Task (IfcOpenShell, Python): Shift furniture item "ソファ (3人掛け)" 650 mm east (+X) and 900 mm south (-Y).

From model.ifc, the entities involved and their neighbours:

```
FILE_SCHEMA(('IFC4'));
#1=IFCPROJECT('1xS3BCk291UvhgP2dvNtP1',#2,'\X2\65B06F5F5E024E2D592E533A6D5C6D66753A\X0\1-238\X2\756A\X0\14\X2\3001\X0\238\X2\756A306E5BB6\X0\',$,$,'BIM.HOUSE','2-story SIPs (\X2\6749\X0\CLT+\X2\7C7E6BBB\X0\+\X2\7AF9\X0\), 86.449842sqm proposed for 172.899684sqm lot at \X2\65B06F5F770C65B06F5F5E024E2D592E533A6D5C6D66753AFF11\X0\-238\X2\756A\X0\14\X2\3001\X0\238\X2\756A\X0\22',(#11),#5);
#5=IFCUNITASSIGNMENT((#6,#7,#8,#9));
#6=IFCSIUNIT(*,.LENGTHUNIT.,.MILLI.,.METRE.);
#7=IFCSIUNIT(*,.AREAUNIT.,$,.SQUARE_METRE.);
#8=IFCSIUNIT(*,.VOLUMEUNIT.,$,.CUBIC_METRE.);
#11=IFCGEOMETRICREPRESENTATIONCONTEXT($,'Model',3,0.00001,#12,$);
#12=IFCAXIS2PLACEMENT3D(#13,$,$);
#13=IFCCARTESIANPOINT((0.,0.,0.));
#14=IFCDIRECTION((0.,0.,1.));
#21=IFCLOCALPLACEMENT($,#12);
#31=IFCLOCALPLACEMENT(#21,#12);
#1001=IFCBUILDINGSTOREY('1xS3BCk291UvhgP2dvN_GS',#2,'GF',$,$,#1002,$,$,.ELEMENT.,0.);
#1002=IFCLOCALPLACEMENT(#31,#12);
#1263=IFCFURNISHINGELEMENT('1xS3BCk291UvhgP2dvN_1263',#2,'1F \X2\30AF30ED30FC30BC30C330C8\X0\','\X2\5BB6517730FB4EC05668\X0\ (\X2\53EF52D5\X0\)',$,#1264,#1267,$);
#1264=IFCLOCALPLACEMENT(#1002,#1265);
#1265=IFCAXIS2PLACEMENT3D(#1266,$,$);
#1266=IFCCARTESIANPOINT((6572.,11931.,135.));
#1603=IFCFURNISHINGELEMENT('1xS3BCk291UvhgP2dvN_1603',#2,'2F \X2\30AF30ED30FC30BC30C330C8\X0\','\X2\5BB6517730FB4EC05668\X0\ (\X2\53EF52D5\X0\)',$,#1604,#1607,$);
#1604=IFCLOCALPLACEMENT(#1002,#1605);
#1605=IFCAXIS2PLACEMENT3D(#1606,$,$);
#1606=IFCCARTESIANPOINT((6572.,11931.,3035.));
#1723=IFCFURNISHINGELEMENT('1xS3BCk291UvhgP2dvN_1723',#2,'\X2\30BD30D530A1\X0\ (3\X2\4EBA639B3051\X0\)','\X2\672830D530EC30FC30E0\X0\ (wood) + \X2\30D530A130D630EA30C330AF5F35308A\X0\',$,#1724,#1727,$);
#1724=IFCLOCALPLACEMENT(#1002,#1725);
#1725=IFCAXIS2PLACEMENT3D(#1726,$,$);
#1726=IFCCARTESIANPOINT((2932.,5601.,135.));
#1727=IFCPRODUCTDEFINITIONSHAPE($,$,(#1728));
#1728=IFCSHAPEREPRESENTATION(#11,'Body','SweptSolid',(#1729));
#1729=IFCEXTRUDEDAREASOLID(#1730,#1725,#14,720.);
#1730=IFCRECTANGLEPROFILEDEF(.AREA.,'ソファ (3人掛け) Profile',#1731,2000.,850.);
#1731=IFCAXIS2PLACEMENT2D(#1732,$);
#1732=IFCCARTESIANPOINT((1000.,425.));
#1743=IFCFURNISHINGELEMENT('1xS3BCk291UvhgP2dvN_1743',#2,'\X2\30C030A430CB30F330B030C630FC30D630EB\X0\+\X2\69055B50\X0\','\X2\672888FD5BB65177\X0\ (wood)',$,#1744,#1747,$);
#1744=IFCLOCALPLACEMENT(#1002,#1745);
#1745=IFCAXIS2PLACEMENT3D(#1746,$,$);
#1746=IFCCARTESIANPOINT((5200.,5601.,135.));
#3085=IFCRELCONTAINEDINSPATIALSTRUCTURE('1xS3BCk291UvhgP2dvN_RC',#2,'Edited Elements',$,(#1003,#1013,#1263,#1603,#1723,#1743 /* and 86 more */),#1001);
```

```python
import ifcopenshell
import ifcopenshell.api.geometry
import ifcopenshell.util.placement

model = ifcopenshell.open("model.ifc")

item = model.by_id(1723)
matrix = ifcopenshell.util.placement.get_local_placement(item.ObjectPlacement)
matrix[0, 3] += 650.0
matrix[1, 3] -= 900.0
ifcopenshell.api.geometry.edit_object_placement(model, product=item, matrix=matrix, is_si=False)

print(ifcopenshell.util.placement.get_local_placement(item.ObjectPlacement).round(3) + 0.0)

model.write("model-out.ifc")
```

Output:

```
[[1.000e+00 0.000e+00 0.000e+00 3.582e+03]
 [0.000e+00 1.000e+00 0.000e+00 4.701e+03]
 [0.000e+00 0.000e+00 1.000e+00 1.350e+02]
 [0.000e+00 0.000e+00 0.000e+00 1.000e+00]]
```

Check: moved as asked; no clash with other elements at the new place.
